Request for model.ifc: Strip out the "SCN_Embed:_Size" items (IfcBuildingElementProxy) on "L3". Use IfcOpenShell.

First a look at what the model holds.

```python
import ifcopenshell
import ifcopenshell.util.element

model = ifcopenshell.open("model.ifc")
print(model.schema)
storey = next(s for s in model.by_type("IfcBuildingStorey") if s.Name == "L3")
proxies = [e for e in ifcopenshell.util.element.get_decomposition(storey) if e.is_a("IfcBuildingElementProxy")]
seen = {}
for e in proxies:
    element_type = ifcopenshell.util.element.get_type(e)
    name = element_type.Name if element_type not in (None, e) else None
    seen[name] = seen.get(name, 0) + 1
for name, count in sorted(seen.items(), key=str):
    print(count, "x", name)
```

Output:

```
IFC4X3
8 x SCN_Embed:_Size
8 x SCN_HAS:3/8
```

```python
import ifcopenshell
import ifcopenshell.api.root
import ifcopenshell.util.element

model = ifcopenshell.open("model.ifc")

storey = next(s for s in model.by_type("IfcBuildingStorey") if s.Name == "L3")
proxies = [e for e in ifcopenshell.util.element.get_decomposition(storey) if e.is_a("IfcBuildingElementProxy")]
targets = [e for e in proxies if (t := ifcopenshell.util.element.get_type(e)) not in (None, e) and t.Name == "SCN_Embed:_Size"]

for e in targets:
    ifcopenshell.api.root.remove_product(model, product=e)
print(len(targets), "removed")

model.write("model_rev.ifc")
```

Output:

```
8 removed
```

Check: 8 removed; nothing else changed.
